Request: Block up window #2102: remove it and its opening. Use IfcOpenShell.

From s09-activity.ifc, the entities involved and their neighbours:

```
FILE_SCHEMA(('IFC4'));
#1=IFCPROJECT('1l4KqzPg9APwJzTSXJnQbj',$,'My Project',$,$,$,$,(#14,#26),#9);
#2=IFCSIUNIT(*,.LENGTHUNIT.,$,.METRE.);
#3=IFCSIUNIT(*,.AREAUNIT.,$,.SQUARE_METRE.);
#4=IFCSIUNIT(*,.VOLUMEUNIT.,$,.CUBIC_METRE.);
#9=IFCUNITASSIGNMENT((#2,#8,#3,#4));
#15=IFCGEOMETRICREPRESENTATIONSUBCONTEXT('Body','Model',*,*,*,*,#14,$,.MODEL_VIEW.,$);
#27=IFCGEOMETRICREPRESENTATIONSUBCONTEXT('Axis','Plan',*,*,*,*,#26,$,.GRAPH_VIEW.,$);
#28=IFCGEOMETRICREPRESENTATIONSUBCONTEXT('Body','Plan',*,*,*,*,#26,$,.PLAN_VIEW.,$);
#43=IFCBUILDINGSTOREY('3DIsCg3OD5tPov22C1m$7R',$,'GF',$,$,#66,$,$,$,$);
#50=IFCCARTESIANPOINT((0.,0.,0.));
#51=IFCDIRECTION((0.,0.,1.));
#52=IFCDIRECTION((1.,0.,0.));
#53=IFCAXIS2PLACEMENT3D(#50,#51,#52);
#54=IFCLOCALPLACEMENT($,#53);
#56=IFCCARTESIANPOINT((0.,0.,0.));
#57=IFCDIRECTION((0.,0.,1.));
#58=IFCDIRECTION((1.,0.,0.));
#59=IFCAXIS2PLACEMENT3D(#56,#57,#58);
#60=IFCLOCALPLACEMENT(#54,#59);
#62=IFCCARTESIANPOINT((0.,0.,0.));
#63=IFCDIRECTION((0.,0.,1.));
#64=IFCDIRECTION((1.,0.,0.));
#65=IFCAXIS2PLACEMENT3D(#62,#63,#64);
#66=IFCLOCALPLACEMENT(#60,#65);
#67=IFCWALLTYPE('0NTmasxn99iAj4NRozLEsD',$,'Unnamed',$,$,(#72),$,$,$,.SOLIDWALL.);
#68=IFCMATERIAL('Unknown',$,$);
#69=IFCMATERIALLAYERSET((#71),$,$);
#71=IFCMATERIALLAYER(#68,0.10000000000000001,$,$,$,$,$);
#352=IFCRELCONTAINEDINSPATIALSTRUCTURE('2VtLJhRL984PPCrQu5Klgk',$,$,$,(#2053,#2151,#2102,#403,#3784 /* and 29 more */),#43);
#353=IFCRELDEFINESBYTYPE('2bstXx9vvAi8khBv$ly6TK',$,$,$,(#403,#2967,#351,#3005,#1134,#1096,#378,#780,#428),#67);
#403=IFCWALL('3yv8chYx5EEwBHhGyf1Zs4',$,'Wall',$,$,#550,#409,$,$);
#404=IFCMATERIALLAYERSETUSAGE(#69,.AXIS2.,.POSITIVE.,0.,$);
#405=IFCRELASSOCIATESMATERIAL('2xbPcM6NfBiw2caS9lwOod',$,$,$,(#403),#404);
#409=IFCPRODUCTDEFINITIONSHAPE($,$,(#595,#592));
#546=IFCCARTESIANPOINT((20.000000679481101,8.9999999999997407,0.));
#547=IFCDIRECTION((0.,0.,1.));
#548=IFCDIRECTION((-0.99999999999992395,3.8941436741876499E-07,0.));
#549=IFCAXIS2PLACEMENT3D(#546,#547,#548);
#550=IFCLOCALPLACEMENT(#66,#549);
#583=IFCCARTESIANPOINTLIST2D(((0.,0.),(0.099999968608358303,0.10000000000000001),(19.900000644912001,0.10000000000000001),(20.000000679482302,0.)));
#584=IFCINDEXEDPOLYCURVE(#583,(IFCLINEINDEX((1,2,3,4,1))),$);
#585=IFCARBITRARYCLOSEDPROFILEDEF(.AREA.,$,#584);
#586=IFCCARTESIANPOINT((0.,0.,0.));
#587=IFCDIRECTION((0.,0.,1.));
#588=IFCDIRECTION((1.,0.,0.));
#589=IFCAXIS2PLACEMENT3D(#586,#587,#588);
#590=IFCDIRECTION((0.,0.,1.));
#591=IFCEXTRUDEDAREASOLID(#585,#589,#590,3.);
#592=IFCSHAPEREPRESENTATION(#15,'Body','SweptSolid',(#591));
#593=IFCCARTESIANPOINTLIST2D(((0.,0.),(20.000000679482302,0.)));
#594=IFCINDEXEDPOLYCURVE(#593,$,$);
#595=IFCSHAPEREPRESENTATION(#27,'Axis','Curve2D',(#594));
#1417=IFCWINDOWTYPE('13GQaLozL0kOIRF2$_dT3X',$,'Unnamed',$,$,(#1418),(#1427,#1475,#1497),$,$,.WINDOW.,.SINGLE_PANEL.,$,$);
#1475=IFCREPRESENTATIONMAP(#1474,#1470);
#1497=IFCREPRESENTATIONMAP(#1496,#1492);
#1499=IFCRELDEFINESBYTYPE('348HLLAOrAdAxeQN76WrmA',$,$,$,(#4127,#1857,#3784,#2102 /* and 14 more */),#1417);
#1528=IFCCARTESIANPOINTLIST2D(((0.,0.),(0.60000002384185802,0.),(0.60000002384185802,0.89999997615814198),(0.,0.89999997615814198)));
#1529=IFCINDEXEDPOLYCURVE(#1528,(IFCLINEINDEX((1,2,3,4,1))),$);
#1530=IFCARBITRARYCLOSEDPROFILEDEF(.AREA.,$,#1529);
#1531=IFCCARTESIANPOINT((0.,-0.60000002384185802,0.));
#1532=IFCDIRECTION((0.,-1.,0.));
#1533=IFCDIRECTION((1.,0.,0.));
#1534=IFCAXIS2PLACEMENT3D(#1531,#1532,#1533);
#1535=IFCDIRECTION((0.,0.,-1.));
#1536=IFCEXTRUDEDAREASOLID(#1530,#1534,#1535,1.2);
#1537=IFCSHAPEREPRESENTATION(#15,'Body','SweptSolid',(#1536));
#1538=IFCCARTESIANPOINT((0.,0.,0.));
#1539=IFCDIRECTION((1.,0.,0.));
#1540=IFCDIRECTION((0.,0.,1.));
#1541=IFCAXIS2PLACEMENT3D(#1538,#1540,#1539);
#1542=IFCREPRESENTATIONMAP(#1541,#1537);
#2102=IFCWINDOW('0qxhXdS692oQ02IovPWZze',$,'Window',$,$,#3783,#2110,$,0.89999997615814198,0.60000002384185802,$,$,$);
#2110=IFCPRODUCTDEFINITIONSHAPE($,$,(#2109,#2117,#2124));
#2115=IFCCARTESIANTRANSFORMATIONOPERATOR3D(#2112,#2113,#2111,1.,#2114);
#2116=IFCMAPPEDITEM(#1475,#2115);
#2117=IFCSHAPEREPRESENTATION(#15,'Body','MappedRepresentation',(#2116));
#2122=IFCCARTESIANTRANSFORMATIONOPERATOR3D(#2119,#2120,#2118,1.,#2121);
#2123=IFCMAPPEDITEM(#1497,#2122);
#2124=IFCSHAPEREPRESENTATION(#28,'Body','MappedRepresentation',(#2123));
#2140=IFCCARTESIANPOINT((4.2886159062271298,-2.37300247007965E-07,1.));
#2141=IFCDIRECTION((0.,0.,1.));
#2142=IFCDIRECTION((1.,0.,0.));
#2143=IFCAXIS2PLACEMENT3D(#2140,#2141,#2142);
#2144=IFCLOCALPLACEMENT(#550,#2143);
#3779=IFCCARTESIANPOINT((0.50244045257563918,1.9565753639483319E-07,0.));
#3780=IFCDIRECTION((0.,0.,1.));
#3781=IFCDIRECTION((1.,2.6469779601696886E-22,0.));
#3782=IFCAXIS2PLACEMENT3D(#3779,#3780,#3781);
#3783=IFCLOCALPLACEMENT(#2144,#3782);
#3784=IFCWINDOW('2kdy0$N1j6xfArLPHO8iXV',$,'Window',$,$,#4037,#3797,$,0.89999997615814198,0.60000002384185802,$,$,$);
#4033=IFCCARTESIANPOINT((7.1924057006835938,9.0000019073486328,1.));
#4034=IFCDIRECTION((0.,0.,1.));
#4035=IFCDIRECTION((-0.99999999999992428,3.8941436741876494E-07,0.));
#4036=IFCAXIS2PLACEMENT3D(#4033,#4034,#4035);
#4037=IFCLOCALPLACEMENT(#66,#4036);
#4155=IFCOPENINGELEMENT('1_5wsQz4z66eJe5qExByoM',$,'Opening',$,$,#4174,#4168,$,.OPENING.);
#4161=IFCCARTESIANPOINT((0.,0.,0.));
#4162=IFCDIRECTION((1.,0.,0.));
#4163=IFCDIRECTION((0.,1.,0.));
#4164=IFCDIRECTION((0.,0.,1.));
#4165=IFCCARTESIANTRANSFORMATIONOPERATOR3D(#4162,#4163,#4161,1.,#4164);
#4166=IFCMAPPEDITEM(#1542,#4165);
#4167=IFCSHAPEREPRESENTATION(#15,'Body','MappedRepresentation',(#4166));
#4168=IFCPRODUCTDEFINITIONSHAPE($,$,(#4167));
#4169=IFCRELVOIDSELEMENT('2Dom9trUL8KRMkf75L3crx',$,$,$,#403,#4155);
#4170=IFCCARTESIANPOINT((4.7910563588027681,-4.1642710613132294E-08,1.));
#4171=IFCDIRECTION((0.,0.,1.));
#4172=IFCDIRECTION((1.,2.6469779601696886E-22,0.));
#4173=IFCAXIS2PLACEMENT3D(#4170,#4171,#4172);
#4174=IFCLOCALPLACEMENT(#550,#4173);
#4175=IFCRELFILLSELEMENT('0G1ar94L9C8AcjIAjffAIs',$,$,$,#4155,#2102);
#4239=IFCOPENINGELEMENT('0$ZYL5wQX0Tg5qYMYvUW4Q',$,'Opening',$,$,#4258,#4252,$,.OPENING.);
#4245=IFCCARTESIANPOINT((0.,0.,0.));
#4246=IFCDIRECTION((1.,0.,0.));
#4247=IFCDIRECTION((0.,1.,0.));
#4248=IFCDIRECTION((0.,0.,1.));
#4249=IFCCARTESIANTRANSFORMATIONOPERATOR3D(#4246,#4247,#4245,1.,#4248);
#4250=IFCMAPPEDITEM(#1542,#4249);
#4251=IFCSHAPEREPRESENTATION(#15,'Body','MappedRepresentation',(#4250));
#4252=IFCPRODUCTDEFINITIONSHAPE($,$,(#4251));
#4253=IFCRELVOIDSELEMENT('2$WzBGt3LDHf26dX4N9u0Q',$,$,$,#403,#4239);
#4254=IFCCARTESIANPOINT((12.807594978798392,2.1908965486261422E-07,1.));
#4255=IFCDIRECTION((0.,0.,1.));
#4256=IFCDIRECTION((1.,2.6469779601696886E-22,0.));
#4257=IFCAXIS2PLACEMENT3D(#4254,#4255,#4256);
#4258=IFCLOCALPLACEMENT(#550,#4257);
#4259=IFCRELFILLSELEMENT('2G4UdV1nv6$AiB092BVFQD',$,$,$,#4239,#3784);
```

```python
import ifcopenshell
import ifcopenshell.api.feature
import ifcopenshell.api.root
import ifcopenshell.geom
import ifcopenshell.util.shape

model = ifcopenshell.open("s09-activity.ifc")
settings = ifcopenshell.geom.settings()


def volume(element):
    """Net volume in cubic metres, openings subtracted."""
    shape = ifcopenshell.geom.create_shape(settings, element)
    return ifcopenshell.util.shape.get_volume(shape.geometry)


window = model.by_id(2102)
opening = window.FillsVoids[0].RelatingOpeningElement
wall = opening.VoidsElements[0].RelatingBuildingElement
before = volume(wall)

ifcopenshell.api.root.remove_product(model, product=window)
ifcopenshell.api.feature.remove_feature(model, feature=opening)

after = volume(wall)

print(f"wall volume {before:.3f} -> {after:.3f} m3")

model.write("s09-activity_edited.ifc")
```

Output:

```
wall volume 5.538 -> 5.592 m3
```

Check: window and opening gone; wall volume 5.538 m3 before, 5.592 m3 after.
